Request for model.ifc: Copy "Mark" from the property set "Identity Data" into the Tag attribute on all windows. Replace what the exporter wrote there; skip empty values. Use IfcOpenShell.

First a look at what the model holds.

```python
import ifcopenshell
import ifcopenshell.util.element

model = ifcopenshell.open("model.ifc")
print(model.schema)
windows = model.by_type("IfcWindow")
print(len(windows), "windows")
for e in windows[:8]:
    source = ifcopenshell.util.element.get_pset(e, "Identity Data", "Mark")
    target = e.Tag
    print(e.id(), repr(source), repr(target), sep=" | ")
```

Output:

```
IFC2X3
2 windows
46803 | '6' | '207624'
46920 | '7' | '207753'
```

```python
import ifcopenshell
import ifcopenshell.util.element

model = ifcopenshell.open("model.ifc")

count = 0
for e in model.by_type("IfcWindow"):
    value = ifcopenshell.util.element.get_pset(e, "Identity Data", "Mark")
    current = e.Tag
    if not value or not value.strip() or current == value:
        continue
    e.Tag = value
    count += 1

print(count, "windows updated")

model.write("model_v2.ifc")
```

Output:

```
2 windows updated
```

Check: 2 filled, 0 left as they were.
